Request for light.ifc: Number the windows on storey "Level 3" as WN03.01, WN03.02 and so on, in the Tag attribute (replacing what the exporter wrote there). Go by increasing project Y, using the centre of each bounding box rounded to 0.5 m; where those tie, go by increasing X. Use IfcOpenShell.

First a look at what the model holds.

```python
import ifcopenshell
import ifcopenshell.util.element
import ifcopenshell.util.placement

model = ifcopenshell.open("light.ifc")
print(model.schema)
storey = next(s for s in model.by_type("IfcBuildingStorey") if s.Name == "Level 3")
windows = [e for e in ifcopenshell.util.element.get_decomposition(storey) if e.is_a("IfcWindow")]
for e in sorted(windows, key=lambda e: e.id()):
    origin = ifcopenshell.util.placement.get_local_placement(e.ObjectPlacement)[:3, 3]
    print(e.id(), e.Tag, e.Name, origin.round(2) + 0.0, sep=" | ")
```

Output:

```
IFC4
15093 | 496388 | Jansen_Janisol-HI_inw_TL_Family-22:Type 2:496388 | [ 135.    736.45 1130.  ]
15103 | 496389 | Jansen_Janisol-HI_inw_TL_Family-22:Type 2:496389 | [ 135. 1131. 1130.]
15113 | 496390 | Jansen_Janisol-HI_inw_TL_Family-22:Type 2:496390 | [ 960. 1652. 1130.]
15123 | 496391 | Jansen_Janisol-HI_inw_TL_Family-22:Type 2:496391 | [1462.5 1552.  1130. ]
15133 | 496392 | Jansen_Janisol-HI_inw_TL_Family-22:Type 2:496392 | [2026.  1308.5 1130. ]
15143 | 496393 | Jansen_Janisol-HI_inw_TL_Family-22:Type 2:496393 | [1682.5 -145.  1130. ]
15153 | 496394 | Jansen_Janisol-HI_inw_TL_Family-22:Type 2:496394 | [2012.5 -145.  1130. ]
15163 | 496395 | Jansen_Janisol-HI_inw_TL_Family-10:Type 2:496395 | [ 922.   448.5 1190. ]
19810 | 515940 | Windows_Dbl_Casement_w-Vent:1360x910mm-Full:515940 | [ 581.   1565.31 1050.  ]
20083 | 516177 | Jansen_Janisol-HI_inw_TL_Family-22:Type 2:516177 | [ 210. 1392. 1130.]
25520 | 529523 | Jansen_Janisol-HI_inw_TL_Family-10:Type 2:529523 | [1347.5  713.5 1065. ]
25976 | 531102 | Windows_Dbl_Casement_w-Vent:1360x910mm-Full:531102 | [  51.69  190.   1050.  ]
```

```python
import ifcopenshell
import ifcopenshell.geom
import ifcopenshell.util.element
import ifcopenshell.util.shape

model = ifcopenshell.open("light.ifc")
settings = ifcopenshell.geom.settings()
settings.set("use-world-coords", True)


def centre(element):
    shape = ifcopenshell.geom.create_shape(settings, element)
    return ifcopenshell.util.shape.get_bbox_centroid(shape.geometry)


storey = next(s for s in model.by_type("IfcBuildingStorey") if s.Name == "Level 3")
windows = [e for e in ifcopenshell.util.element.get_decomposition(storey) if e.is_a("IfcWindow")]

# Insertion points can sit at a corner or the storey origin, so sort by the geometry (in metres).
centres = {e: centre(e) for e in windows}
windows.sort(key=lambda e: (round(centres[e][1] / 0.5), centres[e][0]))

for i, e in enumerate(windows, start=1):
    number = f"WN03.{i:02d}"
    e.Tag = number
    print(e.id(), number)

model.write("light_updated.ifc")
```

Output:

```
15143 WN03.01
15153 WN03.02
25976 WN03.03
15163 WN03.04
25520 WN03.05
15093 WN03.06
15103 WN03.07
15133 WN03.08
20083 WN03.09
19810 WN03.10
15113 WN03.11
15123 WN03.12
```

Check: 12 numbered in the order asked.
